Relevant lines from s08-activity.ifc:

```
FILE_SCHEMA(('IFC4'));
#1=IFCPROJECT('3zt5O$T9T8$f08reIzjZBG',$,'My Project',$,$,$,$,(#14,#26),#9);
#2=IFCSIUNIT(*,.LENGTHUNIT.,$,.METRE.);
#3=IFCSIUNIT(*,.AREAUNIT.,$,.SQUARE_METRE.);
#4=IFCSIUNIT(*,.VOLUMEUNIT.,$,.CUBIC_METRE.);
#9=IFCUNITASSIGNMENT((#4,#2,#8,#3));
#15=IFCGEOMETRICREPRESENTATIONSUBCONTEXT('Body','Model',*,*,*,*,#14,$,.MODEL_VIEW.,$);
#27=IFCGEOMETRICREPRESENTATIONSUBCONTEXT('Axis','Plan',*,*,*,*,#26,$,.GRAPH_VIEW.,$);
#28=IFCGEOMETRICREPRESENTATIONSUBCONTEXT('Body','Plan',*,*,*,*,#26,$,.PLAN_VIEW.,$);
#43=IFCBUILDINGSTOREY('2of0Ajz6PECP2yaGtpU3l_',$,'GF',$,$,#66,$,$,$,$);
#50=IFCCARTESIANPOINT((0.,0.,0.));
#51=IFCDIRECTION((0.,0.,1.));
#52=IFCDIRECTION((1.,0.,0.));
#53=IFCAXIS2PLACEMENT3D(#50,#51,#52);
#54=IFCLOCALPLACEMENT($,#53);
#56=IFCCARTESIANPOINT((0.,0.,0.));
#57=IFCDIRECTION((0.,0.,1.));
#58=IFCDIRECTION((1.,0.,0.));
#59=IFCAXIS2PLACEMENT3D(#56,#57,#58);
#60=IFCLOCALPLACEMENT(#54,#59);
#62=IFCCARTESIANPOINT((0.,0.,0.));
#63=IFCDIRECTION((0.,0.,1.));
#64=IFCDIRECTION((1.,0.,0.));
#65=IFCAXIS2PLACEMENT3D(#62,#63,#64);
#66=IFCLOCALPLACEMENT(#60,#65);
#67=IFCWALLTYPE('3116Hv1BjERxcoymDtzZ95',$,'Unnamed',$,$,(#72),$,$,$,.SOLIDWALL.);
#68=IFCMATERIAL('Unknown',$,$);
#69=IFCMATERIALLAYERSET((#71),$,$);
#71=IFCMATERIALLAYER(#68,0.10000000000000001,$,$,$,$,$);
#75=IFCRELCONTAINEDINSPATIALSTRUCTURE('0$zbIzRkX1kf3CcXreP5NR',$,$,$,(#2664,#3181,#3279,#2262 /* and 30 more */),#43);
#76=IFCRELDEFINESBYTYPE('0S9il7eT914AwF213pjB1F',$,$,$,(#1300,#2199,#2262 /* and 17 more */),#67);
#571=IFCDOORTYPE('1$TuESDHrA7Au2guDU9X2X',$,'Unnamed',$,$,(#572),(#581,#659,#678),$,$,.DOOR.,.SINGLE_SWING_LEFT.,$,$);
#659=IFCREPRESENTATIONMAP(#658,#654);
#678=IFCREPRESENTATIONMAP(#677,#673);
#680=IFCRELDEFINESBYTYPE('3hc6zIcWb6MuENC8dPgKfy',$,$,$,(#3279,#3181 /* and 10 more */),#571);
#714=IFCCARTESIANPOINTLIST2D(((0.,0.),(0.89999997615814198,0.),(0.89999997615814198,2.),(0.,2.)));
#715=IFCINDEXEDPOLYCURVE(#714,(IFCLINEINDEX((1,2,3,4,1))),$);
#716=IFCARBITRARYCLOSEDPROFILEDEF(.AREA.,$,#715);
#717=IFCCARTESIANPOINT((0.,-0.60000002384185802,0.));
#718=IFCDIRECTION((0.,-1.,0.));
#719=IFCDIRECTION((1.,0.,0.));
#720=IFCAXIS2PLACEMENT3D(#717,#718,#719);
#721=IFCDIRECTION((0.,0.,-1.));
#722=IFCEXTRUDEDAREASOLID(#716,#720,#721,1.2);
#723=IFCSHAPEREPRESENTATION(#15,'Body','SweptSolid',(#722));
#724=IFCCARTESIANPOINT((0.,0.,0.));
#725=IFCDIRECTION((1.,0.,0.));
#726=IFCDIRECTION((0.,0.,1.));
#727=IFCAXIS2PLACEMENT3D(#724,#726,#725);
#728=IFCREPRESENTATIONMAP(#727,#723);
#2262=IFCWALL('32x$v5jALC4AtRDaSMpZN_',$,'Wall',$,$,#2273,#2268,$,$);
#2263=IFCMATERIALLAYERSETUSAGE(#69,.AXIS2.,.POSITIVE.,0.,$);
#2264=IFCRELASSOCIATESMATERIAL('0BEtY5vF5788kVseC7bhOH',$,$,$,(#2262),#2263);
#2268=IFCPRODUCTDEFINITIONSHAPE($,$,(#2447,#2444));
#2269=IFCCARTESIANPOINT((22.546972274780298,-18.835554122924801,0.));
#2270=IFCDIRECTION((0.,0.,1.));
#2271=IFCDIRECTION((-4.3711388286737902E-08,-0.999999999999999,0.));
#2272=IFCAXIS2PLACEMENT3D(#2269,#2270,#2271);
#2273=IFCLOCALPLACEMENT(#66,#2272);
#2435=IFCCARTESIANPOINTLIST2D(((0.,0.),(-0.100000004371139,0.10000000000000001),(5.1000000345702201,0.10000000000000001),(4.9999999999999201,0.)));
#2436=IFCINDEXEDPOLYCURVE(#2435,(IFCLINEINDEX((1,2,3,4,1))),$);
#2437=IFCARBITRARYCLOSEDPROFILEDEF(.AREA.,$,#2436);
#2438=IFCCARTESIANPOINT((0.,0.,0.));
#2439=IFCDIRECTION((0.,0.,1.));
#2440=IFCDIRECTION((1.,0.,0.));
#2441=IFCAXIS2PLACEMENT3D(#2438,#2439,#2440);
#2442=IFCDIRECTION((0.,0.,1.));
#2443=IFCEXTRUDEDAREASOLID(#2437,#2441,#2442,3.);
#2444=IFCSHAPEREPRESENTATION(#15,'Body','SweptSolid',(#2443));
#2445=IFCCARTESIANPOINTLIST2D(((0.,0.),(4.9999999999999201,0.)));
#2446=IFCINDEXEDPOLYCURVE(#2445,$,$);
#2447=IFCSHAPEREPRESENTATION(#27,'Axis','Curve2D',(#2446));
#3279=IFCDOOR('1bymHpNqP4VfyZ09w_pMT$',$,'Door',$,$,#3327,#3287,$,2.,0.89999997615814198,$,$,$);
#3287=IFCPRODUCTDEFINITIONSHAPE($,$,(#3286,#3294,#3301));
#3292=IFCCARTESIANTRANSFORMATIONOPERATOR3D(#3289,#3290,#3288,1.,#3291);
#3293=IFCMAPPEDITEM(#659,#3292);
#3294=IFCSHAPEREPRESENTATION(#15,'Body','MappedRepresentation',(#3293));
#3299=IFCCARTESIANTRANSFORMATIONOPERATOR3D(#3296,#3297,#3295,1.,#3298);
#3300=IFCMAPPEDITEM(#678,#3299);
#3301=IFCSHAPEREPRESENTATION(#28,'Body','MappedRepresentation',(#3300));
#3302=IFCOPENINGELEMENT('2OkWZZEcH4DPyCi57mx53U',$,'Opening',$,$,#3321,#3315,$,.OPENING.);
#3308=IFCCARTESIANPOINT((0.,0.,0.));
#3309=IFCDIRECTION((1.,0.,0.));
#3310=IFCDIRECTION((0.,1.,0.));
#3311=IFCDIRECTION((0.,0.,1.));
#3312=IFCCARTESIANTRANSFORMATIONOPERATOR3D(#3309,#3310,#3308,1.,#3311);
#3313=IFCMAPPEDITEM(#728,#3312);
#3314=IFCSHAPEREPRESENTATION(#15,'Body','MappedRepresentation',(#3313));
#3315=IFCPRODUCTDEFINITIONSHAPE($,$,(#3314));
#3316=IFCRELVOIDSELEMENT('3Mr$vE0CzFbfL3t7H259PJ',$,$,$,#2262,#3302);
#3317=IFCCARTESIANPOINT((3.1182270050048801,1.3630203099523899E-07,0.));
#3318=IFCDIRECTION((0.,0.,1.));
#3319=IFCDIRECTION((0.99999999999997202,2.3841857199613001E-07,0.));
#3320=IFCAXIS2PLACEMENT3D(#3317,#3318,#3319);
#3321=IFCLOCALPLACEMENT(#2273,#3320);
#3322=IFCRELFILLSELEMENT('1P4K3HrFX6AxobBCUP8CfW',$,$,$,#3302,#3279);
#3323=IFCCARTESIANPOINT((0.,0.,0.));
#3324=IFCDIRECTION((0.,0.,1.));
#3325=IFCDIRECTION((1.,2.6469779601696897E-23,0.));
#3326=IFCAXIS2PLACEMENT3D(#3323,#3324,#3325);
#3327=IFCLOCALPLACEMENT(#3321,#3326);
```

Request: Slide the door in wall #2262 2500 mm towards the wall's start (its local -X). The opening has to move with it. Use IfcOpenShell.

```python
import ifcopenshell
import ifcopenshell.api.geometry
import ifcopenshell.util.placement
import ifcopenshell.util.unit

model = ifcopenshell.open("s08-activity.ifc")
unit_scale = ifcopenshell.util.unit.calculate_unit_scale(model)

door = model.by_guid("1bymHpNqP4VfyZ09w_pMT$")
opening = door.FillsVoids[0].RelatingOpeningElement
wall = opening.VoidsElements[0].RelatingBuildingElement

wall_matrix = ifcopenshell.util.placement.get_local_placement(wall.ObjectPlacement)
shift = wall_matrix[:3, 0] * -2.5 / unit_scale
before = ifcopenshell.util.placement.get_local_placement(door.ObjectPlacement)[:3, 3].copy()

# The door is placed relative to its opening, so it follows when the opening moves.
matrix = ifcopenshell.util.placement.get_local_placement(opening.ObjectPlacement)
matrix[:3, 3] += shift
ifcopenshell.api.geometry.edit_object_placement(
    model, product=opening, matrix=matrix, is_si=False, should_transform_children=True
)

after = ifcopenshell.util.placement.get_local_placement(door.ObjectPlacement)[:3, 3]
print("door moved by", (after - before).round(3) + 0.0)

model.write("s08-activity-out.ifc")
```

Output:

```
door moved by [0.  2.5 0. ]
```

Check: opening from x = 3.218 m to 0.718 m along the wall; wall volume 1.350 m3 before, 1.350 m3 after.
